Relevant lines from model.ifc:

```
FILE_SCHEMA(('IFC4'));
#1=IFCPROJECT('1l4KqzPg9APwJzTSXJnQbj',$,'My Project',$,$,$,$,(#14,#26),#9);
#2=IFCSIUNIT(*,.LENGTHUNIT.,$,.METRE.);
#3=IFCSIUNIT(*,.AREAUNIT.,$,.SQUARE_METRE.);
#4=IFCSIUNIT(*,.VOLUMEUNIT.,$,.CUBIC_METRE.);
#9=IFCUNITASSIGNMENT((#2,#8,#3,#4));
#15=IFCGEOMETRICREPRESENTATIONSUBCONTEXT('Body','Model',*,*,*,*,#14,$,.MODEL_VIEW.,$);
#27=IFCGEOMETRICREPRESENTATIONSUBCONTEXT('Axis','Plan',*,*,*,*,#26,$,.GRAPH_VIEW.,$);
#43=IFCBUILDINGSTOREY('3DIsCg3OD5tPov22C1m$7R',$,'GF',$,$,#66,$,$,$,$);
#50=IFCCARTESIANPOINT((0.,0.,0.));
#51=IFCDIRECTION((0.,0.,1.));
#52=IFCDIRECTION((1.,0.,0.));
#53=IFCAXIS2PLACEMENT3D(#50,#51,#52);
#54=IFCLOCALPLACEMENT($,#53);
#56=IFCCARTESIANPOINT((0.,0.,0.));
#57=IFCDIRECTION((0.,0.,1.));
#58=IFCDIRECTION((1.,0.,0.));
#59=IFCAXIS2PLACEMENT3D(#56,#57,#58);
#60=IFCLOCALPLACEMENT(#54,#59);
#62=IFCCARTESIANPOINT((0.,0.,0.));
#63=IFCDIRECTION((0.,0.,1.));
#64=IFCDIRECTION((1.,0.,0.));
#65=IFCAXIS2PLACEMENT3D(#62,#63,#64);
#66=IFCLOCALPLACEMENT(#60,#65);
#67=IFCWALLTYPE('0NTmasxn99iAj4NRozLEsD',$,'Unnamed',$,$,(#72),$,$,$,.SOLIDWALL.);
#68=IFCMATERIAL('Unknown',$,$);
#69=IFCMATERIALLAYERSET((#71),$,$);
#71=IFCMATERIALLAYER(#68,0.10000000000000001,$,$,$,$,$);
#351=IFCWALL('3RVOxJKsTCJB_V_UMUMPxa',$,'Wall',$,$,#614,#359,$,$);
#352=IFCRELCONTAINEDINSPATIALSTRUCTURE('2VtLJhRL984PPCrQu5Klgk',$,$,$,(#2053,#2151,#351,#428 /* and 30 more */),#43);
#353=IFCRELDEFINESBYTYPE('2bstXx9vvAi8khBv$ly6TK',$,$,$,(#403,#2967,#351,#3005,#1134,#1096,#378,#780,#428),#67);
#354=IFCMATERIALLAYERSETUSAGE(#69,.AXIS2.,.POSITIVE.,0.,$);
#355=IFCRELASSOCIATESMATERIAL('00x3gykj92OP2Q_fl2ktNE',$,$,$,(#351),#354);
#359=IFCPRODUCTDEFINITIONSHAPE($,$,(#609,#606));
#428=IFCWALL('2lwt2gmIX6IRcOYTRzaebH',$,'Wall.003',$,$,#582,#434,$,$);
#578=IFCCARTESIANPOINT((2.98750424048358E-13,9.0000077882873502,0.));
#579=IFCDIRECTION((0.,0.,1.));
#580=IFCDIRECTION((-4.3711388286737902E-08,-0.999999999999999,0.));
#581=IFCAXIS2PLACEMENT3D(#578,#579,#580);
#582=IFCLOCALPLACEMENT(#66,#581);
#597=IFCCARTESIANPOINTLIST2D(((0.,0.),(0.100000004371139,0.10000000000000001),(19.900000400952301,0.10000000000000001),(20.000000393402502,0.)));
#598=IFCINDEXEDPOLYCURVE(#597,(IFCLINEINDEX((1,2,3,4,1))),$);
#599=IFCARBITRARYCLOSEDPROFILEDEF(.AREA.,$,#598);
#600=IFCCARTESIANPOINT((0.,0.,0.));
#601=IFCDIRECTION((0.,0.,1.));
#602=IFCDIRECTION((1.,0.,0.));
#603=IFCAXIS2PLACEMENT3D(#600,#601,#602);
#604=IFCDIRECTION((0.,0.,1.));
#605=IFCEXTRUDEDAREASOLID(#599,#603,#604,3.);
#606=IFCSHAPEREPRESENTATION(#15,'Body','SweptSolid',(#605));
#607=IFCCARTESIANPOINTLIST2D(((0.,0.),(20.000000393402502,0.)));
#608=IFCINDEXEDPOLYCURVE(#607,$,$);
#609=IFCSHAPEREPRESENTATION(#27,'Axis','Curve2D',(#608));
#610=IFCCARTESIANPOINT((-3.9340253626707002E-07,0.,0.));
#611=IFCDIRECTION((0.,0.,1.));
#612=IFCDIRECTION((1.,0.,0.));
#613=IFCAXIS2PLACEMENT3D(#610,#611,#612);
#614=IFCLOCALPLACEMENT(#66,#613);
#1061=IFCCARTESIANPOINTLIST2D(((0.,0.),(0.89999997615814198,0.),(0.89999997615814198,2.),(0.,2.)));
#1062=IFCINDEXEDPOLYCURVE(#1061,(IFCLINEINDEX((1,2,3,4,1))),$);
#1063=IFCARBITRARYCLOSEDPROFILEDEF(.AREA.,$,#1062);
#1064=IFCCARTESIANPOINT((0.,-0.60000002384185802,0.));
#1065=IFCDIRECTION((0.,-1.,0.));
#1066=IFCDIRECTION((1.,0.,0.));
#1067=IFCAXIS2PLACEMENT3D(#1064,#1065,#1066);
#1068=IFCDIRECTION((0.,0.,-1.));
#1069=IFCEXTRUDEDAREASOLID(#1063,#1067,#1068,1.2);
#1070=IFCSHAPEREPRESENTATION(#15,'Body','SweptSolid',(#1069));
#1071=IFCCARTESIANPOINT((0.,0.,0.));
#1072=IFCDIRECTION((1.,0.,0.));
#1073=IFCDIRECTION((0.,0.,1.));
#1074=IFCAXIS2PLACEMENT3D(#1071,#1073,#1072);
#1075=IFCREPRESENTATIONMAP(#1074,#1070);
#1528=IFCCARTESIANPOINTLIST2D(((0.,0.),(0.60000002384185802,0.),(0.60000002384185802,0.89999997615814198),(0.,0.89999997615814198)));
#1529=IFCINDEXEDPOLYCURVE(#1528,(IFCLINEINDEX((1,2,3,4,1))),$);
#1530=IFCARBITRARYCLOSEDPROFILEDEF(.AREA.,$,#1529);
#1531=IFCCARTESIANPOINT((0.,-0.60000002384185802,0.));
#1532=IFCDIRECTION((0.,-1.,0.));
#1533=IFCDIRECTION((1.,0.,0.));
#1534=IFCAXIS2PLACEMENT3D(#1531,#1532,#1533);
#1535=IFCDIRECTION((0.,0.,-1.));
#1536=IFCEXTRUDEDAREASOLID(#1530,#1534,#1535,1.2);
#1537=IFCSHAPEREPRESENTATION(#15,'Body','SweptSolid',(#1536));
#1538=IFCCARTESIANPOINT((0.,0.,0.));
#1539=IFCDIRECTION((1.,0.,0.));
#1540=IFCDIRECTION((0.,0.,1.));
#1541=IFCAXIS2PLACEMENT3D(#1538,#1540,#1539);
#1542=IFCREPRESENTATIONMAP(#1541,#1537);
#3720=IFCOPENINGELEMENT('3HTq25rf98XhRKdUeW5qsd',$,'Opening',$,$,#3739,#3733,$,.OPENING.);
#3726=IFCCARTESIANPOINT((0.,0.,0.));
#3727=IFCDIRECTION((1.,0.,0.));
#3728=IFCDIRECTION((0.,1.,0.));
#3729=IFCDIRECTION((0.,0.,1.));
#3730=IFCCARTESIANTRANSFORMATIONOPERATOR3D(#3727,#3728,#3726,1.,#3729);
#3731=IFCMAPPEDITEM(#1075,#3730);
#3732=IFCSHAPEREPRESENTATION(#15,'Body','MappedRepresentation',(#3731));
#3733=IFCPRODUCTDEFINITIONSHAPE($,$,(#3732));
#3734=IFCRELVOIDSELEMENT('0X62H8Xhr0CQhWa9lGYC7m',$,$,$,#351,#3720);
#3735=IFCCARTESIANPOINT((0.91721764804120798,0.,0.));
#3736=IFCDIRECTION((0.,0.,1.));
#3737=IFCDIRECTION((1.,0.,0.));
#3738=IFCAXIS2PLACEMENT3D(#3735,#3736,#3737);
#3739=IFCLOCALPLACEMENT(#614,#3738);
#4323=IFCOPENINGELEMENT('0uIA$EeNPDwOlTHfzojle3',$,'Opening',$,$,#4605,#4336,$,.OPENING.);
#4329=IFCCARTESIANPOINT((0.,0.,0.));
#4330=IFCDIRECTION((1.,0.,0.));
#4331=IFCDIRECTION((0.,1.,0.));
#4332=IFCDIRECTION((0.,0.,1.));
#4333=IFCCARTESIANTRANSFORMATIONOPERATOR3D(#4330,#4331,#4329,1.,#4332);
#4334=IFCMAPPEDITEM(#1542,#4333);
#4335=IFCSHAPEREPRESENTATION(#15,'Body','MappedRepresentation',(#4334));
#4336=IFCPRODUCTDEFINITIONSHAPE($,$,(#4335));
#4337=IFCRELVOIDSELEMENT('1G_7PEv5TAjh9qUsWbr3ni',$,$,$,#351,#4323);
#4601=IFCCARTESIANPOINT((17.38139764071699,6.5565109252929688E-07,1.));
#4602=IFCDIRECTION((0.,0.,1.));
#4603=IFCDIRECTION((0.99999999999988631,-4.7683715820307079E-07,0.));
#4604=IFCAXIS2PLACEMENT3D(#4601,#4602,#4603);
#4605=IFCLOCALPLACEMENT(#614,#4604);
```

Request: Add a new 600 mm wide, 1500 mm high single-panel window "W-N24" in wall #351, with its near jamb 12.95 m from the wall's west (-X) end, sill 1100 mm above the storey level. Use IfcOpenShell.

```python
import numpy as np
import ifcopenshell
import ifcopenshell.api.feature
import ifcopenshell.api.geometry
import ifcopenshell.api.root
import ifcopenshell.api.spatial
import ifcopenshell.geom
import ifcopenshell.util.element
import ifcopenshell.util.placement
import ifcopenshell.util.representation
import ifcopenshell.util.shape
import ifcopenshell.util.unit

model = ifcopenshell.open("model.ifc")
unit_scale = ifcopenshell.util.unit.calculate_unit_scale(model)
settings = ifcopenshell.geom.settings()


def volume(element):
    """Net volume in cubic metres, openings subtracted."""
    shape = ifcopenshell.geom.create_shape(settings, element)
    return ifcopenshell.util.shape.get_volume(shape.geometry)


wall = model.by_guid("3RVOxJKsTCJB_V_UMUMPxa")
storey = ifcopenshell.util.element.get_container(wall, ifc_class="IfcBuildingStorey")
context = ifcopenshell.util.representation.get_context(model, "Model", "Body", "MODEL_VIEW")
before = volume(wall)

width, height, from_end, sill = 0.6, 1.5, 12.95, 1.1  # metres

# The wall runs along its own X axis, and the end named is its -X end.
wall_shape = ifcopenshell.geom.create_shape(settings, wall)
x, y, z = ifcopenshell.util.shape.get_vertices(wall_shape.geometry).T
start = x.min() + from_end
face, thickness = float(y.min()), float(y.max() - y.min())
wall_matrix = ifcopenshell.util.placement.get_local_placement(wall.ObjectPlacement)
level = ifcopenshell.util.placement.get_local_placement(storey.ObjectPlacement)[2, 3]


def in_wall(x, y):
    """Placement at x, y metres in the wall's axes, at sill height."""
    matrix = wall_matrix.copy()
    matrix[:, 3] = wall_matrix @ np.array([x / unit_scale, y / unit_scale, 0.0, 1.0])
    matrix[2, 3] = level + sill / unit_scale
    return matrix


# Opening: a box that overshoots both wall faces by 50 mm.
opening = ifcopenshell.api.root.create_entity(model, ifc_class="IfcOpeningElement", predefined_type="OPENING")
box = ifcopenshell.api.geometry.add_wall_representation(
    model, context=context, length=width, height=height, thickness=thickness + 0.1
)
ifcopenshell.api.geometry.assign_representation(model, product=opening, representation=box)
ifcopenshell.api.geometry.edit_object_placement(model, product=opening, matrix=in_wall(start, face - 0.05), is_si=False)
ifcopenshell.api.feature.add_feature(model, feature=opening, element=wall)

window = ifcopenshell.api.root.create_entity(model, ifc_class="IfcWindow", name="W-N24", predefined_type="WINDOW")
window.OverallWidth, window.OverallHeight = width / unit_scale, height / unit_scale
window.PartitioningType = "SINGLE_PANEL"
body = ifcopenshell.api.geometry.add_window_representation(
    model,
    context=context,
    overall_width=window.OverallWidth,
    overall_height=window.OverallHeight,
    partition_type="SINGLE_PANEL",
)
ifcopenshell.api.geometry.assign_representation(model, product=window, representation=body)
ifcopenshell.api.spatial.assign_container(model, products=[window], relating_structure=storey)
ifcopenshell.api.feature.add_filling(model, opening=opening, element=window)

# Centre the window in the wall's thickness.
ifcopenshell.api.geometry.edit_object_placement(model, product=window, matrix=in_wall(start, face), is_si=False)
window_shape = ifcopenshell.geom.create_shape(settings, window)
depth = ifcopenshell.util.shape.get_vertices(window_shape.geometry)[:, 1]
offset = face + thickness / 2 - (depth.min() + depth.max()) / 2
ifcopenshell.api.geometry.edit_object_placement(model, product=window, matrix=in_wall(start, offset), is_si=False)

after = volume(wall)

print(f"wall volume {before:.3f} -> {after:.3f} m3")

model.write("model_edited.ifc")
```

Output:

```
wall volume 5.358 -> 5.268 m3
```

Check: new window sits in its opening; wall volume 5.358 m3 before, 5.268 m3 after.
